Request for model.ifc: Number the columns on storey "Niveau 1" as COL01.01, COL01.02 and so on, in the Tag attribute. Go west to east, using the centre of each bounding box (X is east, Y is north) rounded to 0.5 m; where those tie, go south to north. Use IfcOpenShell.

First a look at what the model holds.

```python
import ifcopenshell
import ifcopenshell.util.element
import ifcopenshell.util.placement

model = ifcopenshell.open("model.ifc")
print(model.schema)
storey = next(s for s in model.by_type("IfcBuildingStorey") if s.Name == "Niveau 1")
columns = [e for e in ifcopenshell.util.element.get_decomposition(storey) if e.is_a("IfcColumn")]
for e in sorted(columns, key=lambda e: e.id()):
    origin = ifcopenshell.util.placement.get_local_placement(e.ObjectPlacement)[:3, 3]
    print(e.id(), e.Tag, e.Name, origin.round(2) + 0.0, sep=" | ")
```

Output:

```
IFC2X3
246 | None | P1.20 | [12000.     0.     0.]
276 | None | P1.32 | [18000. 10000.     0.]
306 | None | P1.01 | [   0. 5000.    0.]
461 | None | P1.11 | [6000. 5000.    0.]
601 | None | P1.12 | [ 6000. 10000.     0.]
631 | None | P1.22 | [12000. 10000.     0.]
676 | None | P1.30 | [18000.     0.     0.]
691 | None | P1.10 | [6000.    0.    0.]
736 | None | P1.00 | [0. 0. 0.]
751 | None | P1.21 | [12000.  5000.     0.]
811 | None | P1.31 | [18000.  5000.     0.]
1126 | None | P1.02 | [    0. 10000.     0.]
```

```python
import ifcopenshell
import ifcopenshell.geom
import ifcopenshell.util.element
import ifcopenshell.util.shape

model = ifcopenshell.open("model.ifc")
settings = ifcopenshell.geom.settings()
settings.set("use-world-coords", True)


def centre(element):
    shape = ifcopenshell.geom.create_shape(settings, element)
    return ifcopenshell.util.shape.get_bbox_centroid(shape.geometry)


storey = next(s for s in model.by_type("IfcBuildingStorey") if s.Name == "Niveau 1")
columns = [e for e in ifcopenshell.util.element.get_decomposition(storey) if e.is_a("IfcColumn")]

# Insertion points can sit at a corner or the storey origin, so sort by the geometry (in metres).
centres = {e: centre(e) for e in columns}
columns.sort(key=lambda e: (round(centres[e][0] / 0.5), centres[e][1]))

for i, e in enumerate(columns, start=1):
    number = f"COL01.{i:02d}"
    e.Tag = number
    print(e.id(), number)

model.write("model_updated.ifc")
```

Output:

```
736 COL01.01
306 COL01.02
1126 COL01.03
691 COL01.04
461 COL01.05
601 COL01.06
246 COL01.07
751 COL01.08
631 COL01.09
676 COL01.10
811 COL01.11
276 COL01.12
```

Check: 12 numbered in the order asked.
